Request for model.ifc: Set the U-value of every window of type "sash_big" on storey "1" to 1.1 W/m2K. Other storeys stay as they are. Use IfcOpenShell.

First a look at what the model holds.

```python
import ifcopenshell
import ifcopenshell.util.element

model = ifcopenshell.open("model.ifc")
print(model.schema)
storey = next(s for s in model.by_type("IfcBuildingStorey") if s.Name == "1")
windows = [e for e in ifcopenshell.util.element.get_decomposition(storey) if e.is_a("IfcWindow")]
seen = {}
for e in windows:
    element_type = ifcopenshell.util.element.get_type(e)
    key = (element_type.Name if element_type != e and element_type else None, ifcopenshell.util.element.get_pset(e, "Pset_WindowCommon", "ThermalTransmittance"))
    seen[key] = seen.get(key, 0) + 1
for (name, value), count in sorted(seen.items(), key=str):
    print(count, "x", name, "|", value)
```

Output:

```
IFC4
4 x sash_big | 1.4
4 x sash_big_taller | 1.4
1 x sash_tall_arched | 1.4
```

```python
import ifcopenshell
import ifcopenshell.api.pset
import ifcopenshell.util.element

model = ifcopenshell.open("model.ifc")

storey = next(s for s in model.by_type("IfcBuildingStorey") if s.Name == "1")
windows = [e for e in ifcopenshell.util.element.get_decomposition(storey) if e.is_a("IfcWindow")]

count = 0
for e in windows:
    element_type = ifcopenshell.util.element.get_type(e)
    if element_type in (None, e) or element_type.Name != "sash_big":
        continue
    # add_pset returns the element's existing set when there is one.
    pset = ifcopenshell.api.pset.add_pset(model, product=e, name="Pset_WindowCommon")
    ifcopenshell.api.pset.edit_pset(model, pset=pset, properties={"ThermalTransmittance": 1.1})
    count += 1

print(count, "windows updated")

model.write("model_v2.ifc")
```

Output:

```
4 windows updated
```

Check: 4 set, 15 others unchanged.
